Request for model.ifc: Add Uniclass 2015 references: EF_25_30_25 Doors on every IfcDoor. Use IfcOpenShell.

First a look at what the model holds.

```python
import ifcopenshell

model = ifcopenshell.open("model.ifc")
print(model.schema)
print("classifications:", [c.Name for c in model.by_type("IfcClassification")])
for ifc_class in ("IfcDoor", "IfcRoof", "IfcStair", "IfcWall", "IfcWindow"):
    print(ifc_class, len(model.by_type(ifc_class)))
```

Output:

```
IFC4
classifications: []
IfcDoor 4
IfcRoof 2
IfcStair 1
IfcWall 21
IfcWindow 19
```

```python
import ifcopenshell
import ifcopenshell.api.classification

model = ifcopenshell.open("model.ifc")

system = ifcopenshell.api.classification.add_classification(model, classification="Uniclass 2015")

codes = {
    "IfcDoor": ("EF_25_30_25", "Doors"),
}
for ifc_class, (code, name) in codes.items():
    products = model.by_type(ifc_class)
    ifcopenshell.api.classification.add_reference(
        model, products=products, classification=system, identification=code, name=name
    )
    print(code, len(products))

model.write("model_rev.ifc")
```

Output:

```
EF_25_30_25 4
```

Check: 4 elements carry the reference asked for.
